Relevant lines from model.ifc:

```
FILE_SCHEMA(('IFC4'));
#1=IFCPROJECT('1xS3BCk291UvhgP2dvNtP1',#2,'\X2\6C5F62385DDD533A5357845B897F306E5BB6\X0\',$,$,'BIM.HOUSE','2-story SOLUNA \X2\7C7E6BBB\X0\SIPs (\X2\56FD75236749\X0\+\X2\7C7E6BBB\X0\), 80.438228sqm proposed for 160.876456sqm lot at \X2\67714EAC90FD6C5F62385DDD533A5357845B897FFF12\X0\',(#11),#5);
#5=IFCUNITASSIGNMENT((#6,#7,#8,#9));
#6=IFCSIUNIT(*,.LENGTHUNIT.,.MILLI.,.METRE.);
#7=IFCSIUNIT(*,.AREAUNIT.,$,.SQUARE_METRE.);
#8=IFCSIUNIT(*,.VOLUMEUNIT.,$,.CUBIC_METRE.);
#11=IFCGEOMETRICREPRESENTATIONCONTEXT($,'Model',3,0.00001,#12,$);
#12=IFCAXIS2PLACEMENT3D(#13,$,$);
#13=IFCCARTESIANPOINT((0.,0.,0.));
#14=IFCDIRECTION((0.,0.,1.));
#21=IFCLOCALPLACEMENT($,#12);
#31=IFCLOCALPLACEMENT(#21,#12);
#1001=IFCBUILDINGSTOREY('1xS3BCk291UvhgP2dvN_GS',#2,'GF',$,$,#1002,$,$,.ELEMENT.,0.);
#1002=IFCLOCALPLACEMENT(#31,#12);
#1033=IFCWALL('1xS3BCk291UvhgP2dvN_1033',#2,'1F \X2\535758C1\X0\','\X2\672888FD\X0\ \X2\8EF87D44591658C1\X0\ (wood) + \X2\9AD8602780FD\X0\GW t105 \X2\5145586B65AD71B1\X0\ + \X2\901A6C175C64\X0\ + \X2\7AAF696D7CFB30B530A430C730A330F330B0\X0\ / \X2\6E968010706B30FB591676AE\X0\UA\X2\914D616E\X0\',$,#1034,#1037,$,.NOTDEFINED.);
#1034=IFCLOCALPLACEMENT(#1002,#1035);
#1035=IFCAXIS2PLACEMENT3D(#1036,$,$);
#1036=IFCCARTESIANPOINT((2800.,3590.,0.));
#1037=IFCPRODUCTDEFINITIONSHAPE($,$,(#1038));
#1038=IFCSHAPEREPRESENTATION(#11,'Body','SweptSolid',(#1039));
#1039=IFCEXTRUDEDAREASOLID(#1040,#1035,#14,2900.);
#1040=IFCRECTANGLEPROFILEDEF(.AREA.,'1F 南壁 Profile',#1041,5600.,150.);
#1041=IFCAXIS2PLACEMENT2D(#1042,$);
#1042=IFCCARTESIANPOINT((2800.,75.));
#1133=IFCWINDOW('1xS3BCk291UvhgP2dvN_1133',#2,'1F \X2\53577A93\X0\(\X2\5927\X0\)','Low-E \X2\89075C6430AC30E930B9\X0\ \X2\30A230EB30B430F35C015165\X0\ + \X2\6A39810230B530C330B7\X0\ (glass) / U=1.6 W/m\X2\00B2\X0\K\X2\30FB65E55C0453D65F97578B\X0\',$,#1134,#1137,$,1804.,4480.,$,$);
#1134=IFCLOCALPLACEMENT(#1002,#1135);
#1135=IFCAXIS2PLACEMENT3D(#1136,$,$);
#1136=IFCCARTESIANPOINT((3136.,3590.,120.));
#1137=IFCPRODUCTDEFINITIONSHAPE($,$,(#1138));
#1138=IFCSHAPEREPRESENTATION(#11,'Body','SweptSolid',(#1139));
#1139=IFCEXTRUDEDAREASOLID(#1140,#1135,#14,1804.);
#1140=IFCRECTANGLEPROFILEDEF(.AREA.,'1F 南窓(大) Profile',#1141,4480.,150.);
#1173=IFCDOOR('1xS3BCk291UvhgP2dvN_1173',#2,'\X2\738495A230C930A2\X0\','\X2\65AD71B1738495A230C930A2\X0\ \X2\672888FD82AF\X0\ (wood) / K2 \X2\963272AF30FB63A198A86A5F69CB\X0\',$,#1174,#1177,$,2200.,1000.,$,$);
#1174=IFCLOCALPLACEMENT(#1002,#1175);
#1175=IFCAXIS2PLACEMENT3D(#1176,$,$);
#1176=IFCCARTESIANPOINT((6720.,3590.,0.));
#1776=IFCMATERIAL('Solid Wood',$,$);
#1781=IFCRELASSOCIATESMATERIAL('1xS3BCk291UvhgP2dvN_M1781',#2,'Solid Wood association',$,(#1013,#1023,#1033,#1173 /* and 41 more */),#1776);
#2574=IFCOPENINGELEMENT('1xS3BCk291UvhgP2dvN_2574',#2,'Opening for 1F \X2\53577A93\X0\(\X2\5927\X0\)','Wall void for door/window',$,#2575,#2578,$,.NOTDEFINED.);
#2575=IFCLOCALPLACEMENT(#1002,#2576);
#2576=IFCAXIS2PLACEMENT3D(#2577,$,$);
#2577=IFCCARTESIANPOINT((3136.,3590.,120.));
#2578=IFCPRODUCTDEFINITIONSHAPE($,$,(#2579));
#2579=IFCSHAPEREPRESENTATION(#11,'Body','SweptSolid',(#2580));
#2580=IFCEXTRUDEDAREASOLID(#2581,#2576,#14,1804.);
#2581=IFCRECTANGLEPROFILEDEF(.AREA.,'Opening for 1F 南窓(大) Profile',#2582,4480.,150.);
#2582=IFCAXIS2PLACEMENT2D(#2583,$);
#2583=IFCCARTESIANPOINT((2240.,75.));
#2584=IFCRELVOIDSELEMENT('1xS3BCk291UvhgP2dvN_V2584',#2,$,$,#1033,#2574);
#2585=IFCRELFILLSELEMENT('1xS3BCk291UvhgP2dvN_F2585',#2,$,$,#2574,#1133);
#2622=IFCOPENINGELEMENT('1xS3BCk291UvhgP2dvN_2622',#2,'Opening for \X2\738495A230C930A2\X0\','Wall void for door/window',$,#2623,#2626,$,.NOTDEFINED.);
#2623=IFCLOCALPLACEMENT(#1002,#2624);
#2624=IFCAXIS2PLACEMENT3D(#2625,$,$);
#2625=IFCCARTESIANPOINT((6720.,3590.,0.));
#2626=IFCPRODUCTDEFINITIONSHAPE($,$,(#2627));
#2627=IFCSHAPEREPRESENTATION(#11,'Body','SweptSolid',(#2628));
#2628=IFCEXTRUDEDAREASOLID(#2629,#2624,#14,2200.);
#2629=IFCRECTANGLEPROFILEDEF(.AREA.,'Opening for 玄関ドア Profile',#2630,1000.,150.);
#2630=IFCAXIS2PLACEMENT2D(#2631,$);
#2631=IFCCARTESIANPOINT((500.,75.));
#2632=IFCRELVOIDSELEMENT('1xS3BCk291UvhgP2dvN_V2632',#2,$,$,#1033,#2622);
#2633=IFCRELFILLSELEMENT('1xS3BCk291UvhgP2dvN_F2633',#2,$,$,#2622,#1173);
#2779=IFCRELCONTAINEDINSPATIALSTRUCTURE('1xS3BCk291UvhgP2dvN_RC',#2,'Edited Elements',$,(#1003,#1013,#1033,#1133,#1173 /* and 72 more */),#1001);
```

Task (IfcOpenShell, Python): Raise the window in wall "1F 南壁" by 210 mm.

```python
import numpy as np
import ifcopenshell
import ifcopenshell.api.geometry
import ifcopenshell.util.placement
import ifcopenshell.util.unit

model = ifcopenshell.open("model.ifc")
unit_scale = ifcopenshell.util.unit.calculate_unit_scale(model)

window = model.by_guid("1xS3BCk291UvhgP2dvN_1133")
opening = window.FillsVoids[0].RelatingOpeningElement
dz = 210.0

shift = np.array([0.0, 0.0, dz])
# The window is not placed relative to its opening, so move both.
for product in (opening, window):
    matrix = ifcopenshell.util.placement.get_local_placement(product.ObjectPlacement)
    matrix[:3, 3] += shift
    ifcopenshell.api.geometry.edit_object_placement(model, product=product, matrix=matrix, is_si=False)

print(f"moved by {dz * unit_scale:+.3f} m")

model.write("model_v2.ifc")
```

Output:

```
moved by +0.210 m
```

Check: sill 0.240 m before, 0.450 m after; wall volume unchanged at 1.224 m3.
